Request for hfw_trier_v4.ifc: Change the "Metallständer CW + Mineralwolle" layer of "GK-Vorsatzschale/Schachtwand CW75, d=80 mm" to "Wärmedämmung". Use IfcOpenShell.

First a look at what the model holds.

```python
import ifcopenshell
import ifcopenshell.util.element

model = ifcopenshell.open("hfw_trier_v4.ifc")
print(model.schema)
for layer_set in model.by_type("IfcMaterialLayerSet"):
    if layer_set.LayerSetName == "GK-Vorsatzschale/Schachtwand CW75, d=80 mm":
        for layer in layer_set.MaterialLayers:
            print(layer.id(), layer.Material and layer.Material.Name, layer.LayerThickness, sep=" | ")
        print(len(ifcopenshell.util.element.get_elements_by_material(model, layer_set)), "elements and types use it")
print(sorted(m.Name for m in model.by_type("IfcMaterial") if m.Name)[:60])
```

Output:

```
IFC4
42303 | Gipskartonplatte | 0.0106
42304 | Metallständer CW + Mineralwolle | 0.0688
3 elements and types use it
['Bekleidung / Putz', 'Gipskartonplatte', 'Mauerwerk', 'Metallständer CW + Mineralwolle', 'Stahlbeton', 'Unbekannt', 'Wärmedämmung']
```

```python
import ifcopenshell
import ifcopenshell.api.material

model = ifcopenshell.open("hfw_trier_v4.ifc")

layer_set = next(s for s in model.by_type("IfcMaterialLayerSet") if s.LayerSetName == "GK-Vorsatzschale/Schachtwand CW75, d=80 mm")
layer = next(l for l in layer_set.MaterialLayers if l.Material and l.Material.Name == "Metallständer CW + Mineralwolle")
material = next(m for m in model.by_type("IfcMaterial") if m.Name == "Wärmedämmung")

# Point this one layer at the other material; renaming the old one would change it everywhere.
ifcopenshell.api.material.edit_layer(model, layer=layer, attributes={"Name": material.Name}, material=material)

print([l.Material.Name if l.Material else None for l in layer_set.MaterialLayers])

model.write("hfw_trier_v4-out.ifc")
```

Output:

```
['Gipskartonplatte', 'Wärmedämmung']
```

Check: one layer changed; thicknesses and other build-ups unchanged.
